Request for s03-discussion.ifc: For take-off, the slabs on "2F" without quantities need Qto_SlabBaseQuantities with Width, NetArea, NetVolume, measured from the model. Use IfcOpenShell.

First a look at what the model holds.

```python
import ifcopenshell
import ifcopenshell.util.element
import ifcopenshell.util.unit

model = ifcopenshell.open("s03-discussion.ifc")
print(model.schema)
for unit_type in ("LENGTHUNIT", "AREAUNIT", "VOLUMEUNIT"):
    print(unit_type, ifcopenshell.util.unit.calculate_unit_scale(model, unit_type))
storey = next(s for s in model.by_type("IfcBuildingStorey") if s.Name == "2F")
slabs = [e for e in ifcopenshell.util.element.get_decomposition(storey) if e.is_a("IfcSlab")]
for e in sorted(slabs, key=lambda e: e.id()):
    print(e.id(), e.is_a(), e.Name, list(ifcopenshell.util.element.get_psets(e, qtos_only=True)), sep=" | ")
```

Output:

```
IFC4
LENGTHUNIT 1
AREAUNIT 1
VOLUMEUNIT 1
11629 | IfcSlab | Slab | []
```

```python
import ifcopenshell
import ifcopenshell.api.pset
import ifcopenshell.geom
import ifcopenshell.util.element
import ifcopenshell.util.shape
import ifcopenshell.util.unit

model = ifcopenshell.open("s03-discussion.ifc")
unit_scale = ifcopenshell.util.unit.calculate_unit_scale(model)
area_scale = ifcopenshell.util.unit.calculate_unit_scale(model, "AREAUNIT")
volume_scale = ifcopenshell.util.unit.calculate_unit_scale(model, "VOLUMEUNIT")
settings = ifcopenshell.geom.settings()

storey = next(s for s in model.by_type("IfcBuildingStorey") if s.Name == "2F")
slabs = [e for e in ifcopenshell.util.element.get_decomposition(storey) if e.is_a("IfcSlab")]

for e in sorted(slabs, key=lambda e: e.id()):
    if ifcopenshell.util.element.get_psets(e, qtos_only=True, should_inherit=False):
        continue
    # Geometry comes back in metres, in the element's own axes.
    shape = ifcopenshell.geom.create_shape(settings, e)
    values = {
        "Width": ifcopenshell.util.shape.get_z(shape.geometry) / unit_scale,
        "NetArea": ifcopenshell.util.shape.get_footprint_area(shape.geometry) / area_scale,
        "NetVolume": ifcopenshell.util.shape.get_volume(shape.geometry) / volume_scale,
    }
    qto = ifcopenshell.api.pset.add_qto(model, product=e, name="Qto_SlabBaseQuantities")
    ifcopenshell.api.pset.edit_qto(model, qto=qto, properties=values)
    print(e.id(), {k: round(v, 3) for k, v in values.items()})

model.write("s03-discussion-out.ifc")
```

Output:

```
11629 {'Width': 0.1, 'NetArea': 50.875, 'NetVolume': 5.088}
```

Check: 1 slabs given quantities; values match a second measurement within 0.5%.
